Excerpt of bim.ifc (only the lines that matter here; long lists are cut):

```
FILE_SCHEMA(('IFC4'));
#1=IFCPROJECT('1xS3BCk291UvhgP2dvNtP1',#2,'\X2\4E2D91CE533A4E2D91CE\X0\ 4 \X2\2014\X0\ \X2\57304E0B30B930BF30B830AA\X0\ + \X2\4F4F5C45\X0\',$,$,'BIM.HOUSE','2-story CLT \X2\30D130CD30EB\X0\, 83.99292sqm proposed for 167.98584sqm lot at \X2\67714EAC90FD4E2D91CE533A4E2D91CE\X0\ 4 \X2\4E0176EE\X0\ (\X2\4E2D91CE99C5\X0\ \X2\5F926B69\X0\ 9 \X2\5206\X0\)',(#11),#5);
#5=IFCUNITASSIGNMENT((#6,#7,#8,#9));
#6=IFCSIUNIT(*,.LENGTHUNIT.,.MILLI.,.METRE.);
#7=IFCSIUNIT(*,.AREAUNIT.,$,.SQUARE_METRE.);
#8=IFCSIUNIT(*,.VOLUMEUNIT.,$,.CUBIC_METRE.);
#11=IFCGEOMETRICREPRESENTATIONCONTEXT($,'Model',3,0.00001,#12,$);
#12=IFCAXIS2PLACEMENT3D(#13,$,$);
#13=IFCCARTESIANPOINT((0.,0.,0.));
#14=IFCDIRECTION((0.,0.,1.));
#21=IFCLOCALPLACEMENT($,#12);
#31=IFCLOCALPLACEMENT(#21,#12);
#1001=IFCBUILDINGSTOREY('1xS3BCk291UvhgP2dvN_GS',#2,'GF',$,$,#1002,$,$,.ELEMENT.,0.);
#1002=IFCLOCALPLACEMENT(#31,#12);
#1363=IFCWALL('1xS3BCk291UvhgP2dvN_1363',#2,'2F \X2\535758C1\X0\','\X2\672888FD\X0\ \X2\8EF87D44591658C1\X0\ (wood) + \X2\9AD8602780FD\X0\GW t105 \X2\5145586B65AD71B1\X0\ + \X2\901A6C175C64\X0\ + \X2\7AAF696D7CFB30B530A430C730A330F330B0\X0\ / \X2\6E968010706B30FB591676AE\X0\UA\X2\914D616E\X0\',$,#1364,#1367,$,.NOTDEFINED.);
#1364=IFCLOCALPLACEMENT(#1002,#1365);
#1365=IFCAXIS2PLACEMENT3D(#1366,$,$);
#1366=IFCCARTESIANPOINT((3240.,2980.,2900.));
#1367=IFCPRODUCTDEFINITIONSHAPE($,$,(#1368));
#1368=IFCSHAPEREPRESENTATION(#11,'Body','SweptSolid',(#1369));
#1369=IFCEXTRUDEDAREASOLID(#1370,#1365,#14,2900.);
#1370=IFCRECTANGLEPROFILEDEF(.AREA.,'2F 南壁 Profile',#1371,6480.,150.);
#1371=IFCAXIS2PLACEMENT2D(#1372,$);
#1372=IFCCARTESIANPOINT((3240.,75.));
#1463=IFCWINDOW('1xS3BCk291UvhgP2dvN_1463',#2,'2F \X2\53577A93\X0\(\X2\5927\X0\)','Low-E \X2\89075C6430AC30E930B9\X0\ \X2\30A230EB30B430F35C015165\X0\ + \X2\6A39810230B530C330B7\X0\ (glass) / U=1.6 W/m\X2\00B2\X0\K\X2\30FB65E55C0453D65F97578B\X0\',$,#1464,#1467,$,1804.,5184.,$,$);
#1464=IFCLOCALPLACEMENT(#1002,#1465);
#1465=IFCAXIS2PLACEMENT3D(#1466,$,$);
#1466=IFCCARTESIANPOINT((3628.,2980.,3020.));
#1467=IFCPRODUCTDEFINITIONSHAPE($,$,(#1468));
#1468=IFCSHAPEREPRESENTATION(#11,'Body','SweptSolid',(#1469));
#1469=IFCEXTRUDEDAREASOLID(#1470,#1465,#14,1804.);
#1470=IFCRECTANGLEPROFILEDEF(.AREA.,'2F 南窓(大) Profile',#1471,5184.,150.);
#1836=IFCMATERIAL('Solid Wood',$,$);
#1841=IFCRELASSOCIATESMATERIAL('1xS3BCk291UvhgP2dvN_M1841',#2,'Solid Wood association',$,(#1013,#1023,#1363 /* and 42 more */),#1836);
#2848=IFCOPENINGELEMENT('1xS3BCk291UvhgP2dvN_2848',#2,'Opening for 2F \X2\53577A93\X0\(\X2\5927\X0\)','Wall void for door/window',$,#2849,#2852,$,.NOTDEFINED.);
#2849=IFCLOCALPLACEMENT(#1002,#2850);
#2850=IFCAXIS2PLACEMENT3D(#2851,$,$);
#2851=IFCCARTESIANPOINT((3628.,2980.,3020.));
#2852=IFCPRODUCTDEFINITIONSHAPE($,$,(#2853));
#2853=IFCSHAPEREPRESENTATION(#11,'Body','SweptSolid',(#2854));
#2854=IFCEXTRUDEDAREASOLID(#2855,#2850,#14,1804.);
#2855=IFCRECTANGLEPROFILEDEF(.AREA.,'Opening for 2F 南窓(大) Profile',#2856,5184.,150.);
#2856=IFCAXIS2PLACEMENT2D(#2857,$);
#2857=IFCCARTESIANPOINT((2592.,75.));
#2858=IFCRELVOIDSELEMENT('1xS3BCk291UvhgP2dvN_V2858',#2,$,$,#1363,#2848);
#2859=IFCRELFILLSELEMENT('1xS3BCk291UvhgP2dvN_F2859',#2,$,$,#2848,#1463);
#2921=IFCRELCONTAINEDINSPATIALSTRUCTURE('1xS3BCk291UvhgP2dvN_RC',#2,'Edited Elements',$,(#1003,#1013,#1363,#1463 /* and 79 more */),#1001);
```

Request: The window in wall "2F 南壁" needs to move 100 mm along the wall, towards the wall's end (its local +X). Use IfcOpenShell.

```python
import ifcopenshell
import ifcopenshell.api.geometry
import ifcopenshell.util.placement
import ifcopenshell.util.unit

model = ifcopenshell.open("bim.ifc")
unit_scale = ifcopenshell.util.unit.calculate_unit_scale(model)

window = model.by_guid("1xS3BCk291UvhgP2dvN_1463")
opening = window.FillsVoids[0].RelatingOpeningElement
wall = opening.VoidsElements[0].RelatingBuildingElement

wall_matrix = ifcopenshell.util.placement.get_local_placement(wall.ObjectPlacement)
shift = wall_matrix[:3, 0] * 0.1 / unit_scale
before = ifcopenshell.util.placement.get_local_placement(window.ObjectPlacement)[:3, 3].copy()

# The window is not placed relative to its opening, so move both.
for product in (opening, window):
    matrix = ifcopenshell.util.placement.get_local_placement(product.ObjectPlacement)
    matrix[:3, 3] += shift
    ifcopenshell.api.geometry.edit_object_placement(model, product=product, matrix=matrix, is_si=False)

after = ifcopenshell.util.placement.get_local_placement(window.ObjectPlacement)[:3, 3]
print("window moved by", (after - before).round(3) + 0.0)

model.write("bim_v2.ifc")
```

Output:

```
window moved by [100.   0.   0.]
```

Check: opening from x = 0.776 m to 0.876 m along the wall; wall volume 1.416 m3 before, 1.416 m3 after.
